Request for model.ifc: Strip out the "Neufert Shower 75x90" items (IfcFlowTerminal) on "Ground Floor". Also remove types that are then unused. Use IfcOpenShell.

First a look at what the model holds.

```python
import ifcopenshell
import ifcopenshell.util.element

model = ifcopenshell.open("model.ifc")
print(model.schema)
storey = next(s for s in model.by_type("IfcBuildingStorey") if s.Name == "Ground Floor")
terminals = [e for e in ifcopenshell.util.element.get_decomposition(storey) if e.is_a("IfcFlowTerminal")]
seen = {}
for e in terminals:
    element_type = ifcopenshell.util.element.get_type(e)
    name = element_type.Name if element_type not in (None, e) else None
    seen[name] = seen.get(name, 0) + 1
for name, count in sorted(seen.items(), key=str):
    print(count, "x", name)
```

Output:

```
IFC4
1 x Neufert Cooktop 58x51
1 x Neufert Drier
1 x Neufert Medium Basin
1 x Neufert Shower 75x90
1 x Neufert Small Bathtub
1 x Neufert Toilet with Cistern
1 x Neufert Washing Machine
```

```python
import ifcopenshell
import ifcopenshell.api.root
import ifcopenshell.util.element

model = ifcopenshell.open("model.ifc")

storey = next(s for s in model.by_type("IfcBuildingStorey") if s.Name == "Ground Floor")
terminals = [e for e in ifcopenshell.util.element.get_decomposition(storey) if e.is_a("IfcFlowTerminal")]
targets = [e for e in terminals if (t := ifcopenshell.util.element.get_type(e)) not in (None, e) and t.Name == "Neufert Shower 75x90"]
types = {ifcopenshell.util.element.get_type(e) for e in targets} - {None, *targets}

for e in targets:
    ifcopenshell.api.root.remove_product(model, product=e)
print(len(targets), "removed")

unused = [t for t in types if not ifcopenshell.util.element.get_types(t)]
for t in unused:
    ifcopenshell.api.root.remove_product(model, product=t)
print(len(unused), "unused types removed")

model.write("model_rev.ifc")
```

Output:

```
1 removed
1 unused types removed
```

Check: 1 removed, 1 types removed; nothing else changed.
